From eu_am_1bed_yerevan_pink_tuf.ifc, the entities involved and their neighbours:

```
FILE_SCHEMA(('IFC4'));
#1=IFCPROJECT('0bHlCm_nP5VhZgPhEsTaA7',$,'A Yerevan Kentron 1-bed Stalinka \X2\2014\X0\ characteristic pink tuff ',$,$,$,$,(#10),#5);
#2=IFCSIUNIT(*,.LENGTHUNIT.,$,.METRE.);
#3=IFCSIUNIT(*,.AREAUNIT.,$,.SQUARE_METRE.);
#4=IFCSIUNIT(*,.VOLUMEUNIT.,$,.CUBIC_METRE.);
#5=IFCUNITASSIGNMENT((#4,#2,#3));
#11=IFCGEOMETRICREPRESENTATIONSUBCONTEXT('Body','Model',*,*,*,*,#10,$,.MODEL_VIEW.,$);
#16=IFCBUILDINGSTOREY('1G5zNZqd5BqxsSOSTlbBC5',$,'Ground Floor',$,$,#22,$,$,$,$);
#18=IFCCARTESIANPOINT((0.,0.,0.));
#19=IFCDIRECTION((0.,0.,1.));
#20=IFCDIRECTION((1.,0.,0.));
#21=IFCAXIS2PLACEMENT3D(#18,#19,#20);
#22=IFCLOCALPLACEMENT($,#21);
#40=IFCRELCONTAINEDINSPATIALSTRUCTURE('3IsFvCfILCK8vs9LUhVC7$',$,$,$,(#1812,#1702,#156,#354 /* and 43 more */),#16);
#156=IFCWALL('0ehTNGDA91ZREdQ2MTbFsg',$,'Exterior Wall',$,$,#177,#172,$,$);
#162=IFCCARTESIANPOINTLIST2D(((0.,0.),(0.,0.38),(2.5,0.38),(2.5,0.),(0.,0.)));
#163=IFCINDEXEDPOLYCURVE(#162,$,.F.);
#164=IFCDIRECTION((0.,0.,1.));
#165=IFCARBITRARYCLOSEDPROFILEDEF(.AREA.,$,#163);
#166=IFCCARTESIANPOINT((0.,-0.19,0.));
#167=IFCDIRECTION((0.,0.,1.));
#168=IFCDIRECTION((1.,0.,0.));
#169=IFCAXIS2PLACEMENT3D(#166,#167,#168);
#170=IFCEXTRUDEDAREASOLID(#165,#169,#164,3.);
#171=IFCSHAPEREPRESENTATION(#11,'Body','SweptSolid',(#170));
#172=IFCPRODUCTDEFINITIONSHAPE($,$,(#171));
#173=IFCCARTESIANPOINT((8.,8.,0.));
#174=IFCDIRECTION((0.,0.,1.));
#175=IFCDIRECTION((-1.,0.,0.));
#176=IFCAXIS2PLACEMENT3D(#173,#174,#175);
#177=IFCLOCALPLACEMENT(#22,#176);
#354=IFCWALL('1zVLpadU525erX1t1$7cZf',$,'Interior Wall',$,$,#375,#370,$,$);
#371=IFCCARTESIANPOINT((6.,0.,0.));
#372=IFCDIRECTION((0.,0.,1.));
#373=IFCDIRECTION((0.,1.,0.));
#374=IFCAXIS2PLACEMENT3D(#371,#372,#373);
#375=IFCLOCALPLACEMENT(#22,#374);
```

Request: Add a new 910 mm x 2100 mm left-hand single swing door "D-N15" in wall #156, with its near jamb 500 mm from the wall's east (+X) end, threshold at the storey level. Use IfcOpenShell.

```python
import numpy as np
import ifcopenshell
import ifcopenshell.api.feature
import ifcopenshell.api.geometry
import ifcopenshell.api.root
import ifcopenshell.api.spatial
import ifcopenshell.geom
import ifcopenshell.util.element
import ifcopenshell.util.placement
import ifcopenshell.util.representation
import ifcopenshell.util.shape
import ifcopenshell.util.unit

model = ifcopenshell.open("eu_am_1bed_yerevan_pink_tuf.ifc")
unit_scale = ifcopenshell.util.unit.calculate_unit_scale(model)
settings = ifcopenshell.geom.settings()


def volume(element):
    """Net volume in cubic metres, openings subtracted."""
    shape = ifcopenshell.geom.create_shape(settings, element)
    return ifcopenshell.util.shape.get_volume(shape.geometry)


wall = model.by_id(156)
storey = ifcopenshell.util.element.get_container(wall, ifc_class="IfcBuildingStorey")
context = ifcopenshell.util.representation.get_context(model, "Model", "Body", "MODEL_VIEW")
before = volume(wall)

width, height, from_end, sill = 0.91, 2.1, 0.5, 0.0  # metres

# The wall runs along its own X axis, and the end named is its -X end.
wall_shape = ifcopenshell.geom.create_shape(settings, wall)
x, y, z = ifcopenshell.util.shape.get_vertices(wall_shape.geometry).T
start = x.min() + from_end
face, thickness = float(y.min()), float(y.max() - y.min())
wall_matrix = ifcopenshell.util.placement.get_local_placement(wall.ObjectPlacement)
level = ifcopenshell.util.placement.get_local_placement(storey.ObjectPlacement)[2, 3]


def in_wall(x, y):
    """Placement at x, y metres in the wall's axes, at sill height."""
    matrix = wall_matrix.copy()
    matrix[:, 3] = wall_matrix @ np.array([x / unit_scale, y / unit_scale, 0.0, 1.0])
    matrix[2, 3] = level + sill / unit_scale
    return matrix


# Opening: a box that overshoots both wall faces by 50 mm.
opening = ifcopenshell.api.root.create_entity(model, ifc_class="IfcOpeningElement", predefined_type="OPENING")
box = ifcopenshell.api.geometry.add_wall_representation(
    model, context=context, length=width, height=height, thickness=thickness + 0.1
)
ifcopenshell.api.geometry.assign_representation(model, product=opening, representation=box)
ifcopenshell.api.geometry.edit_object_placement(model, product=opening, matrix=in_wall(start, face - 0.05), is_si=False)
ifcopenshell.api.feature.add_feature(model, feature=opening, element=wall)

door = ifcopenshell.api.root.create_entity(model, ifc_class="IfcDoor", name="D-N15", predefined_type="DOOR")
door.OverallWidth, door.OverallHeight = width / unit_scale, height / unit_scale
door.OperationType = "SINGLE_SWING_LEFT"
body = ifcopenshell.api.geometry.add_door_representation(
    model,
    context=context,
    overall_width=door.OverallWidth,
    overall_height=door.OverallHeight,
    operation_type="SINGLE_SWING_LEFT",
    lining_properties={"LiningDepth": thickness / unit_scale, "ThresholdDepth": thickness / unit_scale},
)
ifcopenshell.api.geometry.assign_representation(model, product=door, representation=body)
ifcopenshell.api.spatial.assign_container(model, products=[door], relating_structure=storey)
ifcopenshell.api.feature.add_filling(model, opening=opening, element=door)

# The lining spans the wall, so the door starts at the wall face.
ifcopenshell.api.geometry.edit_object_placement(model, product=door, matrix=in_wall(start, face), is_si=False)

after = volume(wall)

print(f"wall volume {before:.3f} -> {after:.3f} m3")

model.write("eu_am_1bed_yerevan_pink_tuf-out.ifc")
```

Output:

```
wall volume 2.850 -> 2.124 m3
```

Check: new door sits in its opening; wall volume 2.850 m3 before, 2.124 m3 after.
